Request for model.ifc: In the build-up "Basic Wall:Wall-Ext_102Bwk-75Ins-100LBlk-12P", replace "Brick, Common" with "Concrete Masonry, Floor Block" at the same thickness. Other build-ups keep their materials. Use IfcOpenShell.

First a look at what the model holds.

```python
import ifcopenshell
import ifcopenshell.util.element

model = ifcopenshell.open("model.ifc")
print(model.schema)
for layer_set in model.by_type("IfcMaterialLayerSet"):
    if layer_set.LayerSetName == "Basic Wall:Wall-Ext_102Bwk-75Ins-100LBlk-12P":
        for layer in layer_set.MaterialLayers:
            print(layer.id(), layer.Material and layer.Material.Name, layer.LayerThickness, sep=" | ")
        print(len(ifcopenshell.util.element.get_elements_by_material(model, layer_set)), "elements and types use it")
print(sorted(m.Name for m in model.by_type("IfcMaterial") if m.Name)[:60])
```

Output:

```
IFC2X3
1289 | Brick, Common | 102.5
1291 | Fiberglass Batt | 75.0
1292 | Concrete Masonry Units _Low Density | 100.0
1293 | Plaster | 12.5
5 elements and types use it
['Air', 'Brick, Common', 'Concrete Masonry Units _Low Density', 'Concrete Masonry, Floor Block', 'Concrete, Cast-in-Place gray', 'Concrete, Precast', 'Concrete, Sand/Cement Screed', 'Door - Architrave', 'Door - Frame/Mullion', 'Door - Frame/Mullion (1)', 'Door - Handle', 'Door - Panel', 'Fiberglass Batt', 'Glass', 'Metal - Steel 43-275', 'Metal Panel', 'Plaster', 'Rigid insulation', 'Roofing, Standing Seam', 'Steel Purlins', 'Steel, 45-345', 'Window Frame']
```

```python
import ifcopenshell
import ifcopenshell.api.material

model = ifcopenshell.open("model.ifc")

layer_set = next(s for s in model.by_type("IfcMaterialLayerSet") if s.LayerSetName == "Basic Wall:Wall-Ext_102Bwk-75Ins-100LBlk-12P")
layer = next(l for l in layer_set.MaterialLayers if l.Material and l.Material.Name == "Brick, Common")
material = next(m for m in model.by_type("IfcMaterial") if m.Name == "Concrete Masonry, Floor Block")

# Point this one layer at the other material; renaming the old one would change it everywhere.
ifcopenshell.api.material.edit_layer(model, layer=layer, attributes={}, material=material)

print([l.Material.Name if l.Material else None for l in layer_set.MaterialLayers])

model.write("model_updated.ifc")
```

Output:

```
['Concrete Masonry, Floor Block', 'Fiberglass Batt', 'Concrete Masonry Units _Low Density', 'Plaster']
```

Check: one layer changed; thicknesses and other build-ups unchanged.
